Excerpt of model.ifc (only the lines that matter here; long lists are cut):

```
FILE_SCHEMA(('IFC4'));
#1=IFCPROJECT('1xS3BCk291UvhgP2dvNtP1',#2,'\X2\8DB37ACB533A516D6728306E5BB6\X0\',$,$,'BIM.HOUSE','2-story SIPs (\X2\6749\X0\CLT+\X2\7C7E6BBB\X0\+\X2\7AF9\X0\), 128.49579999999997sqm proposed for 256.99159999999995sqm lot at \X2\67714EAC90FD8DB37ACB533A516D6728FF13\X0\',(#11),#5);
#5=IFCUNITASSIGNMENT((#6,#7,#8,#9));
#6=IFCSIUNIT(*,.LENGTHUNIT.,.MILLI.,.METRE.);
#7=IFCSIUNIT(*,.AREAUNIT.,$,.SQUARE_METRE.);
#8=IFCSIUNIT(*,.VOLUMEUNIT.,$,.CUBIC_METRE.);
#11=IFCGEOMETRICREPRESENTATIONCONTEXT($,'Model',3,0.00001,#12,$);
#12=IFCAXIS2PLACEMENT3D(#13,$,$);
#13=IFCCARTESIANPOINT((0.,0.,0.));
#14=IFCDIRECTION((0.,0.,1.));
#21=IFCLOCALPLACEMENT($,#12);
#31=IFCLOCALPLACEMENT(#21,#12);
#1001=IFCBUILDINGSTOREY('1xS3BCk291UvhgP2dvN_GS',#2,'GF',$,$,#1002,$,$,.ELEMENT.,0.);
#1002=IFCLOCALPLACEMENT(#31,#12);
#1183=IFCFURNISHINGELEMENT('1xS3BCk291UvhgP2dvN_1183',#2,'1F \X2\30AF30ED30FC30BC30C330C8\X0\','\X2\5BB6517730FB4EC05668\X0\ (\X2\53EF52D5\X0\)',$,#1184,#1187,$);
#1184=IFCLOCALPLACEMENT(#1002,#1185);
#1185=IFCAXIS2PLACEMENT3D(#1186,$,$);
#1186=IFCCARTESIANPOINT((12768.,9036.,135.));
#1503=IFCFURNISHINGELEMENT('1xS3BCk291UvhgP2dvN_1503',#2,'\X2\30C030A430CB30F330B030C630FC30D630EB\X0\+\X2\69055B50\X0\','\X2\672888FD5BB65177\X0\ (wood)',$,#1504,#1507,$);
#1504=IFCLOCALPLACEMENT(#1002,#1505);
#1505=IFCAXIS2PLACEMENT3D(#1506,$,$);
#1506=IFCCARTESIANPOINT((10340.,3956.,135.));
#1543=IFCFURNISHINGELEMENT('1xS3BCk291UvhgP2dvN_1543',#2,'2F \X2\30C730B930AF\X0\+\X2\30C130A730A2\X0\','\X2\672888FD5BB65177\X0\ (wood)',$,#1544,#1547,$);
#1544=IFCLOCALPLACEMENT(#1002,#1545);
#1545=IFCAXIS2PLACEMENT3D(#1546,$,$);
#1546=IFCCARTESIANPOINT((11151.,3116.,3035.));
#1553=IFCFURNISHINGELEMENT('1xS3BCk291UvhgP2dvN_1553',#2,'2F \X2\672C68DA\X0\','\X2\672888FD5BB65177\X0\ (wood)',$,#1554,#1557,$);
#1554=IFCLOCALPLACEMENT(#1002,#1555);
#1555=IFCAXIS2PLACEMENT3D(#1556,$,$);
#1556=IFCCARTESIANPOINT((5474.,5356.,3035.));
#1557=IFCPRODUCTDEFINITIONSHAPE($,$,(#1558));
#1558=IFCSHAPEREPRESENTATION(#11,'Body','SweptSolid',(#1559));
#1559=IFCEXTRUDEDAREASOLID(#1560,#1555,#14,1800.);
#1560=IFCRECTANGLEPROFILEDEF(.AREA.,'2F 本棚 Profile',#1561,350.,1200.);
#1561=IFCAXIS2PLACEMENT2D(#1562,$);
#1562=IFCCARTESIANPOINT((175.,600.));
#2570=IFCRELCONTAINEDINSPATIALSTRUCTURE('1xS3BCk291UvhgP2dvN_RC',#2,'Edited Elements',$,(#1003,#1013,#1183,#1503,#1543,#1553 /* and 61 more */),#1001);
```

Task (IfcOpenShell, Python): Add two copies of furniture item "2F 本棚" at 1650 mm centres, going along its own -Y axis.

```python
import ifcopenshell
import ifcopenshell.api.geometry
import ifcopenshell.api.root
import ifcopenshell.util.element
import ifcopenshell.util.placement

model = ifcopenshell.open("model.ifc")


def reuse_history(source, copy):
    """copy_class also copies each property set's owner history, people and application; keep the originals."""
    for rel in copy.IsDefinedBy:
        if rel.is_a("IfcRelDefinesByProperties") and (history := rel.RelatingPropertyDefinition.OwnerHistory):
            rel.RelatingPropertyDefinition.OwnerHistory = source.OwnerHistory
            ifcopenshell.util.element.remove_deep2(model, history)


source = model.by_guid("1xS3BCk291UvhgP2dvN_1553")
base = ifcopenshell.util.placement.get_local_placement(source.ObjectPlacement)
step = -base[:3, 1] * 1650.0

for i in range(1, 3):
    copy = ifcopenshell.api.root.copy_class(model, product=source)
    copy.Representation = ifcopenshell.util.element.copy_deep(
        model, source.Representation, exclude=["IfcGeometricRepresentationContext", "IfcRepresentationMap"]
    )
    reuse_history(source, copy)
    matrix = base.copy()
    matrix[:3, 3] += i * step
    print("added at", matrix[:3, 3].round(3) + 0.0)
    ifcopenshell.api.geometry.edit_object_placement(model, product=copy, matrix=matrix, is_si=False)

model.write("model-out.ifc")
```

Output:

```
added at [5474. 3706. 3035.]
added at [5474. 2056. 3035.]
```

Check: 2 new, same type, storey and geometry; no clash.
